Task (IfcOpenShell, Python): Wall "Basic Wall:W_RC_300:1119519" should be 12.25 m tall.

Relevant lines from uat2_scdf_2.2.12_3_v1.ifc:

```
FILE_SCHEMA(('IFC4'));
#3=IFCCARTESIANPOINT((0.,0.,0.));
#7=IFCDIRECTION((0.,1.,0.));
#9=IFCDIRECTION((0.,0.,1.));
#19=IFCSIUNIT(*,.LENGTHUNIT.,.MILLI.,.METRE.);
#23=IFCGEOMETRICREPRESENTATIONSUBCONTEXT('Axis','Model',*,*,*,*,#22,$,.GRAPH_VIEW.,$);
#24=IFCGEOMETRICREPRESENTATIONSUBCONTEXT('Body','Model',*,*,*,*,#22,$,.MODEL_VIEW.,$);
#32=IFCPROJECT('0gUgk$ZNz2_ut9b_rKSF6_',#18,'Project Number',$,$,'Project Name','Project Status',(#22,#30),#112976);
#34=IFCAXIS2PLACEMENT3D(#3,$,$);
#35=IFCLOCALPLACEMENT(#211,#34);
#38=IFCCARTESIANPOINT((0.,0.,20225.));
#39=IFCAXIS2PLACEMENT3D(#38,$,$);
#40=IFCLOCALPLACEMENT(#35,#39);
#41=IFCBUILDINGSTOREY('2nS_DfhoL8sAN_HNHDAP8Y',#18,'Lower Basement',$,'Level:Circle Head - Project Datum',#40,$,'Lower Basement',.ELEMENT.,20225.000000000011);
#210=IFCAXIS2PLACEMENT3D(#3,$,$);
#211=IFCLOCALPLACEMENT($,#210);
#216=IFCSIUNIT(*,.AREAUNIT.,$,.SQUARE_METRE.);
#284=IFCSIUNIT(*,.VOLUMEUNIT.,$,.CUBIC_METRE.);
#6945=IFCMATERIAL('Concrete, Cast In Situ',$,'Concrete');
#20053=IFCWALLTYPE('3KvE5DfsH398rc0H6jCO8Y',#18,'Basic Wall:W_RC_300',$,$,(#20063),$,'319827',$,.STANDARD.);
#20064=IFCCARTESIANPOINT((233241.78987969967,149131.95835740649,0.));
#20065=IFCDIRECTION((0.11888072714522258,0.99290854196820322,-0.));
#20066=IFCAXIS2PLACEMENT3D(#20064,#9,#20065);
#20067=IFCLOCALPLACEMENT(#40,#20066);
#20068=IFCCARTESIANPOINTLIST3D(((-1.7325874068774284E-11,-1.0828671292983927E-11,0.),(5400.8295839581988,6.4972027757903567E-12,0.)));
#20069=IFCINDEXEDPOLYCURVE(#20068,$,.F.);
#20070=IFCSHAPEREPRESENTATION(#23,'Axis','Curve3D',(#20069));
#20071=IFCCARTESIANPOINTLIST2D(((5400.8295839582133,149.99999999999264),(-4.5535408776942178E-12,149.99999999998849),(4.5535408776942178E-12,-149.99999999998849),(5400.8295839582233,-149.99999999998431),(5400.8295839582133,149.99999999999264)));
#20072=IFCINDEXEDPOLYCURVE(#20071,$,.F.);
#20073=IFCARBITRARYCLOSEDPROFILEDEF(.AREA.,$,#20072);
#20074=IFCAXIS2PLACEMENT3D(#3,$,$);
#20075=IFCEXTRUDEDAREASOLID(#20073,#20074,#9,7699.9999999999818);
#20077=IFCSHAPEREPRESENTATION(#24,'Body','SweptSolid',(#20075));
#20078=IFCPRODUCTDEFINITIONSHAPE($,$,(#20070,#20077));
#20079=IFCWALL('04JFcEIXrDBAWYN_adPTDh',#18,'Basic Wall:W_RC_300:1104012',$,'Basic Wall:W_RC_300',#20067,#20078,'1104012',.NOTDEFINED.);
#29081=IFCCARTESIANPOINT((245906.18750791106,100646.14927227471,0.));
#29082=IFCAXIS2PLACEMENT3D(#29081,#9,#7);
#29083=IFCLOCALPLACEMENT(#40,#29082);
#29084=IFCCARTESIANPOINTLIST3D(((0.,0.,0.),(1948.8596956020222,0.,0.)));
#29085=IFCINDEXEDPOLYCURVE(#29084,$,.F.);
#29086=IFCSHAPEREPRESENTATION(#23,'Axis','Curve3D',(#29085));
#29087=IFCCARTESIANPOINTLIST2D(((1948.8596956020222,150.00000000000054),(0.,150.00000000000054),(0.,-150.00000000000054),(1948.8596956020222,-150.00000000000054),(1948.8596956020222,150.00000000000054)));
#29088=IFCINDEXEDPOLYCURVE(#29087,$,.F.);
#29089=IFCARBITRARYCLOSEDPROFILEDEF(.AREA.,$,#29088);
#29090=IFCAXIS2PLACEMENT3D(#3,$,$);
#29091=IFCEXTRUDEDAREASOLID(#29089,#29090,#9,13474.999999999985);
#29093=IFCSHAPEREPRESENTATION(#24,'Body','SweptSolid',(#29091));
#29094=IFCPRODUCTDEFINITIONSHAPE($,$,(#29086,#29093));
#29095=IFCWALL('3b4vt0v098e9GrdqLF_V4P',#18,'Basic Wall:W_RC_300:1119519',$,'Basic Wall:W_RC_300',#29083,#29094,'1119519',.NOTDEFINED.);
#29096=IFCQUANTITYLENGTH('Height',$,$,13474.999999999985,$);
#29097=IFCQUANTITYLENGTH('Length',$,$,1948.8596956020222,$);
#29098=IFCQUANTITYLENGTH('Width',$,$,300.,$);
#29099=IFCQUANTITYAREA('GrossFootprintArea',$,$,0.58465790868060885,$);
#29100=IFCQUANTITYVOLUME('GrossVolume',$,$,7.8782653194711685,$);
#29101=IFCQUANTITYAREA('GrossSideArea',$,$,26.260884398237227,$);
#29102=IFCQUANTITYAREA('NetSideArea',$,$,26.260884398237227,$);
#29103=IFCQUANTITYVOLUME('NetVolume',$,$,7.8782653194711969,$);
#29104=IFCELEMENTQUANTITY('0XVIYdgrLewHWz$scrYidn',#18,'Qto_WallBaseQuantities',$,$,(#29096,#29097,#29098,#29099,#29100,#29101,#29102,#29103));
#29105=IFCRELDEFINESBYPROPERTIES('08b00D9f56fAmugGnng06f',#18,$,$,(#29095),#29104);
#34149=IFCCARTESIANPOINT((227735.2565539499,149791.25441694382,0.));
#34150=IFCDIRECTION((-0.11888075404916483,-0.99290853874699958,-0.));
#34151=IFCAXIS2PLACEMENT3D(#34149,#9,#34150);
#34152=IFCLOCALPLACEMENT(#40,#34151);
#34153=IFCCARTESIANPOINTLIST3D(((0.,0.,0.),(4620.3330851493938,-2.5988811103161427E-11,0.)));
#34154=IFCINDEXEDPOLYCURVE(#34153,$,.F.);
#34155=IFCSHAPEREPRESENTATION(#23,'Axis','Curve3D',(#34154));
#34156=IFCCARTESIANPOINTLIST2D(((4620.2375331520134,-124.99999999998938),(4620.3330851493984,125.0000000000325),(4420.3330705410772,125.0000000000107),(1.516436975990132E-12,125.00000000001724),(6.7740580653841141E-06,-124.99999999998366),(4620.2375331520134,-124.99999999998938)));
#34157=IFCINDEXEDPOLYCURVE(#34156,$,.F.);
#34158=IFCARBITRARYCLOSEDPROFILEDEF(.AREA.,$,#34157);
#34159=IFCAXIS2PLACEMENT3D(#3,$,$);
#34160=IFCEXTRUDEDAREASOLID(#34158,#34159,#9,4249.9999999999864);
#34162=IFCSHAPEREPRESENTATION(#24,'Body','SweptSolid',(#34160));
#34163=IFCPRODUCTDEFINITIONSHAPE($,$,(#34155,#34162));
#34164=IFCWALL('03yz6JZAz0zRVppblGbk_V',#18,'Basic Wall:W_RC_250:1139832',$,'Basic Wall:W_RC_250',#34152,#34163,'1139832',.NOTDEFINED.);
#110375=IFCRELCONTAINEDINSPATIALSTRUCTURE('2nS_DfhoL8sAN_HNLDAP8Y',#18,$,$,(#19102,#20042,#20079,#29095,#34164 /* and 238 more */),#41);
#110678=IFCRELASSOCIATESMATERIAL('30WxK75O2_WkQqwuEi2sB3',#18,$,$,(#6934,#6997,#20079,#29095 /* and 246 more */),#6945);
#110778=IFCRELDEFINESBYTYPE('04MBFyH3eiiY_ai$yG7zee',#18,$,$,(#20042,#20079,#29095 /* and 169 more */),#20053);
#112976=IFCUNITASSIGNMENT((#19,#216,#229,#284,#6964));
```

```python
import ifcopenshell
import ifcopenshell.api.pset
import ifcopenshell.geom
import ifcopenshell.util.element
import ifcopenshell.util.representation
import ifcopenshell.util.shape
import ifcopenshell.util.unit

model = ifcopenshell.open("uat2_scdf_2.2.12_3_v1.ifc")
unit_scale = ifcopenshell.util.unit.calculate_unit_scale(model)
area_scale = ifcopenshell.util.unit.calculate_unit_scale(model, "AREAUNIT")
volume_scale = ifcopenshell.util.unit.calculate_unit_scale(model, "VOLUMEUNIT")
settings = ifcopenshell.geom.settings()


def volume(element):
    """Net volume in cubic metres, openings subtracted."""
    shape = ifcopenshell.geom.create_shape(settings, element)
    return ifcopenshell.util.shape.get_volume(shape.geometry)


wall = model.by_guid("3b4vt0v098e9GrdqLF_V4P")
before = volume(wall)

body = ifcopenshell.util.representation.get_representation(wall, "Model", "Body")
solid = body.Items[0]
old_height = solid.Depth
solid.Depth = 12250.0
after = volume(wall)
thickness = 0.3  # wall thickness in metres

# Update the stored height, areas and volumes.
qto = model.by_id(ifcopenshell.util.element.get_pset(wall, "Qto_WallBaseQuantities", should_inherit=False)["id"])
ifcopenshell.api.pset.edit_qto(model, qto=qto, properties={
    "Height": solid.Depth,
    "GrossVolume": ifcopenshell.util.element.get_pset(wall, "Qto_WallBaseQuantities", "GrossVolume") * solid.Depth / old_height,
    "GrossSideArea": ifcopenshell.util.element.get_pset(wall, "Qto_WallBaseQuantities", "GrossSideArea") * solid.Depth / old_height,
    "NetSideArea": after / thickness / area_scale,
    "NetVolume": after / volume_scale,
})

print(f"height {old_height:g} -> {solid.Depth:g}, volume {before:.3f} -> {after:.3f} m3")

model.write("uat2_scdf_2.2.12_3_v1_edited.ifc")
```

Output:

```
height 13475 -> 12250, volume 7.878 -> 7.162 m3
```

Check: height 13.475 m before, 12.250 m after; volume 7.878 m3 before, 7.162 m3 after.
